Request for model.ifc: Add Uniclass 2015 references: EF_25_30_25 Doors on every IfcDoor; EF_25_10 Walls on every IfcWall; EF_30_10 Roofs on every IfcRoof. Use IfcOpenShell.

First a look at what the model holds.

```python
import ifcopenshell

model = ifcopenshell.open("model.ifc")
print(model.schema)
print("classifications:", [c.Name for c in model.by_type("IfcClassification")])
for ifc_class in ("IfcDoor", "IfcRoof", "IfcStair", "IfcWall", "IfcWindow"):
    print(ifc_class, len(model.by_type(ifc_class)))
```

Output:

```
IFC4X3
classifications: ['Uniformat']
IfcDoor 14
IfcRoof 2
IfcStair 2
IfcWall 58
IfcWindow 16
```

```python
import ifcopenshell
import ifcopenshell.api.classification

model = ifcopenshell.open("model.ifc")

system = ifcopenshell.api.classification.add_classification(model, classification="Uniclass 2015")

codes = {
    "IfcDoor": ("EF_25_30_25", "Doors"),
    "IfcWall": ("EF_25_10", "Walls"),
    "IfcRoof": ("EF_30_10", "Roofs"),
}
for ifc_class, (code, name) in codes.items():
    products = model.by_type(ifc_class)
    ifcopenshell.api.classification.add_reference(
        model, products=products, classification=system, identification=code, name=name
    )
    print(code, len(products))

model.write("model_updated.ifc")
```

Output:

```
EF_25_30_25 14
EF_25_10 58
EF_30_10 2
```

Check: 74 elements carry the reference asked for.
